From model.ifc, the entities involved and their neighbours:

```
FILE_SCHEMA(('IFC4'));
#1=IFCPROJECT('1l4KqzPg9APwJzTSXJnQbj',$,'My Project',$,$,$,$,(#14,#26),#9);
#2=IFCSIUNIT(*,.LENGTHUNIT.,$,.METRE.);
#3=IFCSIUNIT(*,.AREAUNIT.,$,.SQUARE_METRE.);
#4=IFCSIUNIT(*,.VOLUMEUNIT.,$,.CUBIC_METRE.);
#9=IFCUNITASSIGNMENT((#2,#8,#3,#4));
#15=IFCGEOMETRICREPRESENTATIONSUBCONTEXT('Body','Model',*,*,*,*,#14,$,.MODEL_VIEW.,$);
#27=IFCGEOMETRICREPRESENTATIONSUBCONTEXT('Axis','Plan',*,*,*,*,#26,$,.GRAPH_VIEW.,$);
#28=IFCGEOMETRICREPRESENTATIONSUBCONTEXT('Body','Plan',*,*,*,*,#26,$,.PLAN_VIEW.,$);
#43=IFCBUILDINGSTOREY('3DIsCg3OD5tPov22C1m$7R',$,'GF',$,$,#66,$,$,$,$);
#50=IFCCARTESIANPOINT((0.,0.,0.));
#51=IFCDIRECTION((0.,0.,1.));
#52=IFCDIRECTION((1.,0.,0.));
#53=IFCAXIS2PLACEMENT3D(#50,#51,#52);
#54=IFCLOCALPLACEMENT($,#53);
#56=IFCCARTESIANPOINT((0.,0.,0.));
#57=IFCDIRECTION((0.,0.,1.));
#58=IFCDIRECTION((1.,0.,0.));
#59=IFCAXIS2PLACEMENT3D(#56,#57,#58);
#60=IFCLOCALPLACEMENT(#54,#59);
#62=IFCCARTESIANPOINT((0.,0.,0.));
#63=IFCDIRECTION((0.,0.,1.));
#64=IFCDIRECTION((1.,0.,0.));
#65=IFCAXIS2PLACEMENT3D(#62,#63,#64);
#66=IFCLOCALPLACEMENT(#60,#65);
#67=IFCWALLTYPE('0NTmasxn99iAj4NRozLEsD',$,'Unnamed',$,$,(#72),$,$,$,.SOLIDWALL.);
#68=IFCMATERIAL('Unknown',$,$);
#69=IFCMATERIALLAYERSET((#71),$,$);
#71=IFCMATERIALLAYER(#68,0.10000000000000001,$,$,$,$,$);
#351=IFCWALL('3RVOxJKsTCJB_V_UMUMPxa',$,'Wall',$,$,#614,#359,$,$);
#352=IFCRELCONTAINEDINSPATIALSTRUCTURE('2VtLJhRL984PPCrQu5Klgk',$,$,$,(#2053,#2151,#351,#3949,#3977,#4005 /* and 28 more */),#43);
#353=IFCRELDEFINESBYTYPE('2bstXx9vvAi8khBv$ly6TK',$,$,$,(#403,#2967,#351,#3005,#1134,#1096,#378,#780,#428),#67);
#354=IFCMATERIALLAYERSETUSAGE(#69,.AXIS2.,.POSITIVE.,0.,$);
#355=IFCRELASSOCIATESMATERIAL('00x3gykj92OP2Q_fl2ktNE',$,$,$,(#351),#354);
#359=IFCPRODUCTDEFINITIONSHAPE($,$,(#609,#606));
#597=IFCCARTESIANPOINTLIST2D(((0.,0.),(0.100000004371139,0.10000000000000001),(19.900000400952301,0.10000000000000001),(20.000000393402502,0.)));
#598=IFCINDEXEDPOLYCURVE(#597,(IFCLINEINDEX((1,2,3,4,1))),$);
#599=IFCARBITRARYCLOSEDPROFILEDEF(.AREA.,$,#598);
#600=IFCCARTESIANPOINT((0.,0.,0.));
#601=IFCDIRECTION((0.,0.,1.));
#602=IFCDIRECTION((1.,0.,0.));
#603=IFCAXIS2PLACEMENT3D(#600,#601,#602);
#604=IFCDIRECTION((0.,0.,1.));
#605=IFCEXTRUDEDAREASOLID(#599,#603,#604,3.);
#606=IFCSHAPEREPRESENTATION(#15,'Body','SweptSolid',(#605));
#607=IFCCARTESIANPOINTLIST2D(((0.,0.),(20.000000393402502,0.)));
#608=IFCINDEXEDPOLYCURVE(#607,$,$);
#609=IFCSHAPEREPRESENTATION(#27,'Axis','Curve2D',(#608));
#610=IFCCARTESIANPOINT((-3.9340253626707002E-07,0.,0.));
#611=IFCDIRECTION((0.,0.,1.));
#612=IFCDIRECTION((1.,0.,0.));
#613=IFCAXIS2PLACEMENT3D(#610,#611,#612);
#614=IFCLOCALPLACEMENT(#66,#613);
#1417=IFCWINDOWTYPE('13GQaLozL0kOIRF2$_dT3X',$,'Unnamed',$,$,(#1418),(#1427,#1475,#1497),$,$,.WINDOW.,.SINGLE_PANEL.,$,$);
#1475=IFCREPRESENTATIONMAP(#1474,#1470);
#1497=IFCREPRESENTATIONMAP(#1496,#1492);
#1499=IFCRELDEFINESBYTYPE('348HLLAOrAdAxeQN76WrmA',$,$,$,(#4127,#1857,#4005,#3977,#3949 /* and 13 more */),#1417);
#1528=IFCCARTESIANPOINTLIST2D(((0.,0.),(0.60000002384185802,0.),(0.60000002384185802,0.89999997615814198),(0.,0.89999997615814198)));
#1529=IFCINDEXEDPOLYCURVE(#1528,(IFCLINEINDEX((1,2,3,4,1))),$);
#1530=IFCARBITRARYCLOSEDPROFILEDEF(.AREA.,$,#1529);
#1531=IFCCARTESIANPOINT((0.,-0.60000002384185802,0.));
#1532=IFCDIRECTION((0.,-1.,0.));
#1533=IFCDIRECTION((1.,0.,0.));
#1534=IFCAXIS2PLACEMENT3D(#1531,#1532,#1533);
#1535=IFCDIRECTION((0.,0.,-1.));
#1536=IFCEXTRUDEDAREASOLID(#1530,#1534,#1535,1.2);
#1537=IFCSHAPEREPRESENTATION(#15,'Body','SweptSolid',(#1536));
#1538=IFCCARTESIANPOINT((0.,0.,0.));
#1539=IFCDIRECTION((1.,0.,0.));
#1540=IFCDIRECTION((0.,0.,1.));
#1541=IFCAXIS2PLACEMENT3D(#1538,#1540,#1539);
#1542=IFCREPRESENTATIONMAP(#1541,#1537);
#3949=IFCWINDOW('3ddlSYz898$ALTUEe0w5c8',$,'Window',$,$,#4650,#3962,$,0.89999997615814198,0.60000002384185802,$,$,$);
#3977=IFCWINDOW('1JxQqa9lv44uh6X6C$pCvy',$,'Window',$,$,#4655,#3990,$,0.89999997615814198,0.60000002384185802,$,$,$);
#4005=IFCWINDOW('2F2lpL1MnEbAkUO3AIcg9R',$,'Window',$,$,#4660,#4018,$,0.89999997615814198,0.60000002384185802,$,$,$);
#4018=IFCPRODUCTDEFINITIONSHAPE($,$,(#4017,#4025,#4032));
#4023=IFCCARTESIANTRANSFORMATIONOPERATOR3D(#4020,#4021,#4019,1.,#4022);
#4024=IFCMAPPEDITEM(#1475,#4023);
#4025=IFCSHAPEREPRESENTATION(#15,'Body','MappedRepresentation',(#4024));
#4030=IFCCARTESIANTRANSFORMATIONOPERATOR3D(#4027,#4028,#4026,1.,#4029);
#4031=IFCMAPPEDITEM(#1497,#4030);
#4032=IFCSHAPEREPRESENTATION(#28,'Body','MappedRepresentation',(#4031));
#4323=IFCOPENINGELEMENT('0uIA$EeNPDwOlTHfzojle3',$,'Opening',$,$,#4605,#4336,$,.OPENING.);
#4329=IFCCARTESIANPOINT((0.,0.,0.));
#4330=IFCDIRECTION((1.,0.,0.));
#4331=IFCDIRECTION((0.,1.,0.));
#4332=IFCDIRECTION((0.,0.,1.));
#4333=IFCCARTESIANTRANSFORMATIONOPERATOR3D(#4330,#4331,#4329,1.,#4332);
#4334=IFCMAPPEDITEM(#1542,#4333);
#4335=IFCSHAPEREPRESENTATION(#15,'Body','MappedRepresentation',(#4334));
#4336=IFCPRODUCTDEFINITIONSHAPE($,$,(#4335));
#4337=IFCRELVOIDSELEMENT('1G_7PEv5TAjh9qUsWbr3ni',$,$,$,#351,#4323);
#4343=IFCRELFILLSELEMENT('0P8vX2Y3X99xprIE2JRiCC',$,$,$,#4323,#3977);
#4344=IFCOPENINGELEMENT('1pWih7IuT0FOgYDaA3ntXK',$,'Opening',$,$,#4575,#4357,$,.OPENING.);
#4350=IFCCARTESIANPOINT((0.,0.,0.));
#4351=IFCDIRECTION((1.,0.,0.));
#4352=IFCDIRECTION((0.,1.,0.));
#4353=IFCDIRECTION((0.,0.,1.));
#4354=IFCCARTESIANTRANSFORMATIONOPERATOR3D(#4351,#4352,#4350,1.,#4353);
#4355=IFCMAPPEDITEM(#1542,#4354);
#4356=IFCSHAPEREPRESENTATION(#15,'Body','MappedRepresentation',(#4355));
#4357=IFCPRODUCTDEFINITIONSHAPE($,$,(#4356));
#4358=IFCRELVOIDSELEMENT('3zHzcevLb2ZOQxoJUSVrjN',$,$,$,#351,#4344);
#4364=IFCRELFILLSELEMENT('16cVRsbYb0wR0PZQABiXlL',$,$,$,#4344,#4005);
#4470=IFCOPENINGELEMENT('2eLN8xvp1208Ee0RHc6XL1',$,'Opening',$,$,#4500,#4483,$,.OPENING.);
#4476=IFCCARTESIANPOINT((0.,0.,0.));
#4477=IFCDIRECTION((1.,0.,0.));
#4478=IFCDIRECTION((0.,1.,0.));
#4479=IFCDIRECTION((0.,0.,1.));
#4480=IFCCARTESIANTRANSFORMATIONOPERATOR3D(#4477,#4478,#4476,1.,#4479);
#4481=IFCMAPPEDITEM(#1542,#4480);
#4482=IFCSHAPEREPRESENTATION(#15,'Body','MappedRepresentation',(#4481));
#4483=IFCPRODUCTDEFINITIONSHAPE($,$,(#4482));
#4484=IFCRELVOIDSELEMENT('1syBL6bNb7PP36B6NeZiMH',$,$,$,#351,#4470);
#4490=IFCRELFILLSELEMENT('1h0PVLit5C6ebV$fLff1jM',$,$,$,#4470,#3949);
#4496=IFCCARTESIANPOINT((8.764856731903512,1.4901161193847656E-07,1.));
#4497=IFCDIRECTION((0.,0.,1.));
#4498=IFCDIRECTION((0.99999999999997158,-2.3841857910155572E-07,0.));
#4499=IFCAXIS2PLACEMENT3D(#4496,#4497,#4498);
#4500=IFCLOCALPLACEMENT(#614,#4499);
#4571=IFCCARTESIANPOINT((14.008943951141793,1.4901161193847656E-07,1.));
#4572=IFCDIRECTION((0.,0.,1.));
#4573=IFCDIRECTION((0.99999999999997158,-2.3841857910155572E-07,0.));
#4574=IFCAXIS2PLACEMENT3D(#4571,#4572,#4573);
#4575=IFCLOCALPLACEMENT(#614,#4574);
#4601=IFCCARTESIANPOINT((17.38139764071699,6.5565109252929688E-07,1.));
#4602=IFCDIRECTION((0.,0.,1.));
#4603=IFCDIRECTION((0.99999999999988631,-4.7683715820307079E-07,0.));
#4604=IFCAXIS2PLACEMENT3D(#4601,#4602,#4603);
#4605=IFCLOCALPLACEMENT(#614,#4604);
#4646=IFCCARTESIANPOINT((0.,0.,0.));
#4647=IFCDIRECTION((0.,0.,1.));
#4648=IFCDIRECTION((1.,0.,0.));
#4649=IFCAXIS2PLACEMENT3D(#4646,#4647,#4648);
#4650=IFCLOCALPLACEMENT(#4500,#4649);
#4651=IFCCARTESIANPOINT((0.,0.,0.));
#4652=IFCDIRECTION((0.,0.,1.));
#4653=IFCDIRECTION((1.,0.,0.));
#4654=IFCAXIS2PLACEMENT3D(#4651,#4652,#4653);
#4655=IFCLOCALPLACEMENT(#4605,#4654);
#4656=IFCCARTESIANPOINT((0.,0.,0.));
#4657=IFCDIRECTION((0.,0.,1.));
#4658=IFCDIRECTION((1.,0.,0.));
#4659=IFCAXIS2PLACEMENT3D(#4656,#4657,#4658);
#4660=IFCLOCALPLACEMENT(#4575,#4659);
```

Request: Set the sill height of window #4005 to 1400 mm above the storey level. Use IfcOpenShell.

```python
import numpy as np
import ifcopenshell
import ifcopenshell.api.geometry
import ifcopenshell.geom
import ifcopenshell.util.element
import ifcopenshell.util.placement
import ifcopenshell.util.shape
import ifcopenshell.util.unit

model = ifcopenshell.open("model.ifc")
unit_scale = ifcopenshell.util.unit.calculate_unit_scale(model)

window = model.by_guid("2F2lpL1MnEbAkUO3AIcg9R")
opening = window.FillsVoids[0].RelatingOpeningElement
storey = ifcopenshell.util.element.get_container(window, ifc_class="IfcBuildingStorey")
level = ifcopenshell.util.placement.get_local_placement(storey.ObjectPlacement)[2, 3]

# The opening's origin need not be at the sill, so measure its lowest point.
shape = ifcopenshell.geom.create_shape(ifcopenshell.geom.settings(), opening)
bottom = ifcopenshell.util.shape.get_shape_bottom_elevation(shape, shape.geometry) / unit_scale
dz = level + 1.4 / unit_scale - bottom

shift = np.array([0.0, 0.0, dz])
# The window is placed relative to its opening, so it follows when the opening moves.
matrix = ifcopenshell.util.placement.get_local_placement(opening.ObjectPlacement)
matrix[:3, 3] += shift
ifcopenshell.api.geometry.edit_object_placement(
    model, product=opening, matrix=matrix, is_si=False, should_transform_children=True
)

print(f"moved by {dz * unit_scale:+.3f} m")

model.write("model_v2.ifc")
```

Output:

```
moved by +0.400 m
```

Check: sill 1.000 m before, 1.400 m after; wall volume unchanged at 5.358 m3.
